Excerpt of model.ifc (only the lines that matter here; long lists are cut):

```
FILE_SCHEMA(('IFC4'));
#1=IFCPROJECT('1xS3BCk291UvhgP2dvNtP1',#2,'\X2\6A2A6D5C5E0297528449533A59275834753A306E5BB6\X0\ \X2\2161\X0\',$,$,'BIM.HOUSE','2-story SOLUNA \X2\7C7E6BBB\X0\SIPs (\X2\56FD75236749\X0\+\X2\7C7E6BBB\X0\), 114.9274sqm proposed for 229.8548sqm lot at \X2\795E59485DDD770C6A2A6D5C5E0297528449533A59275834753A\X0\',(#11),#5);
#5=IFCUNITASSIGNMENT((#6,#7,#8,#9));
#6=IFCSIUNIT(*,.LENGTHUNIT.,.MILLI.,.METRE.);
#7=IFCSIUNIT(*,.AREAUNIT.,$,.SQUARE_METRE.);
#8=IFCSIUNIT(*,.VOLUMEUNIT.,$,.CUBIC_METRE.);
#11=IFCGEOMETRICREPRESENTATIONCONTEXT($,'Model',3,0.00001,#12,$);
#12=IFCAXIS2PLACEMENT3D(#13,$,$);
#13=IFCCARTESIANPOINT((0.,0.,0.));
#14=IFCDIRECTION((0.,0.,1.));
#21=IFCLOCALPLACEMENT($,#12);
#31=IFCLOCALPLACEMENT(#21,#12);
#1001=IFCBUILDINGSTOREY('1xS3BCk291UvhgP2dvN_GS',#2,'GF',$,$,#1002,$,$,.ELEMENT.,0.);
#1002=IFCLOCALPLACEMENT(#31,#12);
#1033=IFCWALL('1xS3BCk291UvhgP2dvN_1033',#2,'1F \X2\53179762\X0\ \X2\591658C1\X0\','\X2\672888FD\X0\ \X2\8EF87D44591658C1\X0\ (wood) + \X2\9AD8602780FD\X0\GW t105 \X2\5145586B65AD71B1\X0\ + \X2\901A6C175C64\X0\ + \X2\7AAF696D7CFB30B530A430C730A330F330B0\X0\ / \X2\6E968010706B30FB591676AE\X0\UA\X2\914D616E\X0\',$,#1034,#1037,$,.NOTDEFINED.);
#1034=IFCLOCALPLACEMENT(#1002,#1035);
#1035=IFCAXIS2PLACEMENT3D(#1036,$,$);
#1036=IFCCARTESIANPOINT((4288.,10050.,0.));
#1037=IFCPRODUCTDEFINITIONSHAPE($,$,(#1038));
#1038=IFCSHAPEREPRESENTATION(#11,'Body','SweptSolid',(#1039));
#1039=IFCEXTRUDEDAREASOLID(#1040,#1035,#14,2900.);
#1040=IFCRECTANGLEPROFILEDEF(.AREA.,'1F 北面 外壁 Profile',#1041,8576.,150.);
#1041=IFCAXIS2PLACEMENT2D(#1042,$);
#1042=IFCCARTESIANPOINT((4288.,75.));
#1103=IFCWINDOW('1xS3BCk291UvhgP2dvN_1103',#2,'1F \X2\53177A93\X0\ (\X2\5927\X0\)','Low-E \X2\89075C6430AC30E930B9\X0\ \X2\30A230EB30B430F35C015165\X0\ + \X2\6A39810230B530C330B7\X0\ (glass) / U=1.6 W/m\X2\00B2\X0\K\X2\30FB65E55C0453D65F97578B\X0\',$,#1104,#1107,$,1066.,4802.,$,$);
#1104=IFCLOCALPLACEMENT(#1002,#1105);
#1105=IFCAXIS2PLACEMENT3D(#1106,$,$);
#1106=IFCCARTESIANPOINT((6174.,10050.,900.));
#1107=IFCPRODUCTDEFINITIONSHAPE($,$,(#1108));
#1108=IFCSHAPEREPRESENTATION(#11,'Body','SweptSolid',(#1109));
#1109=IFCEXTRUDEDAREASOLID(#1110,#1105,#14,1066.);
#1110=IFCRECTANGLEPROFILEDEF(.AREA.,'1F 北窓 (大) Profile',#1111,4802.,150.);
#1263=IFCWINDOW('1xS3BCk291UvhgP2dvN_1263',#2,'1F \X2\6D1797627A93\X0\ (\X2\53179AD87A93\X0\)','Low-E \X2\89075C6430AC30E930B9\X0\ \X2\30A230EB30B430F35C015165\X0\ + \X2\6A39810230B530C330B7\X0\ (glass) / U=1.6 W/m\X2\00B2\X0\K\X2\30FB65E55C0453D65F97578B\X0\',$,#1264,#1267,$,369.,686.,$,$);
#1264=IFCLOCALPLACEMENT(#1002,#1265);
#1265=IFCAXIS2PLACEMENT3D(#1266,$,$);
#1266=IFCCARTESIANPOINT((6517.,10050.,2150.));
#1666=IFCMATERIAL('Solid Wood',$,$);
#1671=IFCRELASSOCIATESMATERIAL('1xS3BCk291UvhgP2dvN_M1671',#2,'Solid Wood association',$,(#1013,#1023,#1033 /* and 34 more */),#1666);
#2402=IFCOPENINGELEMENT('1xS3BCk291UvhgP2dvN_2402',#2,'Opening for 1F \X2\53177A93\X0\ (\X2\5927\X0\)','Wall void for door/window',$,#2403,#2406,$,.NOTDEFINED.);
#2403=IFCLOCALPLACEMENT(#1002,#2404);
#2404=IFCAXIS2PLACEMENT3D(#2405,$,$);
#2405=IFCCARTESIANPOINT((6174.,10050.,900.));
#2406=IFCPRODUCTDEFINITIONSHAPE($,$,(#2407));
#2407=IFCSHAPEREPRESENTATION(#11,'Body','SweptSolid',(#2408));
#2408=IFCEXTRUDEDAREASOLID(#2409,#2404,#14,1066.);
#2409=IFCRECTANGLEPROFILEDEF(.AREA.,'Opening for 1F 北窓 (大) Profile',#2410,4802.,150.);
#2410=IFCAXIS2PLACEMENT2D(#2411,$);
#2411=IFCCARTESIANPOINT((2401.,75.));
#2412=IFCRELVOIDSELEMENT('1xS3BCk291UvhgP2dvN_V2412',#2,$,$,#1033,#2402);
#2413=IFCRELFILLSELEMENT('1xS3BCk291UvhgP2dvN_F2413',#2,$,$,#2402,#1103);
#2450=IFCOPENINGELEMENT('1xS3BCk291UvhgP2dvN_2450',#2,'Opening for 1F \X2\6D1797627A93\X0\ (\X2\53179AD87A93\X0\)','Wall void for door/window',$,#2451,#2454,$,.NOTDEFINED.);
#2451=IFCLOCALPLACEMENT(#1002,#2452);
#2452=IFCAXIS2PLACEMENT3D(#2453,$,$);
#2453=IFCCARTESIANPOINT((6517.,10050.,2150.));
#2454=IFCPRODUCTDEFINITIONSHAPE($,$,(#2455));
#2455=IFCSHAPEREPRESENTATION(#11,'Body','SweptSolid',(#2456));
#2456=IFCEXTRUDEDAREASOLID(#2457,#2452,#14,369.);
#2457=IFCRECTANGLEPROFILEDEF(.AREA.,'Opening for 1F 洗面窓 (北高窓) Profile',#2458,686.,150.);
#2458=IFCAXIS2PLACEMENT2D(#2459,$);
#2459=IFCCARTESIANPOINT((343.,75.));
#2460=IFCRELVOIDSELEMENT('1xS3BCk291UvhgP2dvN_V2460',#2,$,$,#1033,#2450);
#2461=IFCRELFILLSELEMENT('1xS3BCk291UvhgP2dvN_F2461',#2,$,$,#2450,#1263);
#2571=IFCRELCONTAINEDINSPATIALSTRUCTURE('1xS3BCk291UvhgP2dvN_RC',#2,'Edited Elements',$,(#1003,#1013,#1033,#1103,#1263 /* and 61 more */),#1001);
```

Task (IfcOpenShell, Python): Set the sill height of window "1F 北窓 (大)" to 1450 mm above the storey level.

```python
import numpy as np
import ifcopenshell
import ifcopenshell.api.geometry
import ifcopenshell.geom
import ifcopenshell.util.element
import ifcopenshell.util.placement
import ifcopenshell.util.shape
import ifcopenshell.util.unit

model = ifcopenshell.open("model.ifc")
unit_scale = ifcopenshell.util.unit.calculate_unit_scale(model)

window = model.by_guid("1xS3BCk291UvhgP2dvN_1103")
opening = window.FillsVoids[0].RelatingOpeningElement
storey = ifcopenshell.util.element.get_container(window, ifc_class="IfcBuildingStorey")
level = ifcopenshell.util.placement.get_local_placement(storey.ObjectPlacement)[2, 3]

# The opening's origin need not be at the sill, so measure its lowest point.
shape = ifcopenshell.geom.create_shape(ifcopenshell.geom.settings(), opening)
bottom = ifcopenshell.util.shape.get_shape_bottom_elevation(shape, shape.geometry) / unit_scale
dz = level + 1.45 / unit_scale - bottom

shift = np.array([0.0, 0.0, dz])
# The window is not placed relative to its opening, so move both.
for product in (opening, window):
    matrix = ifcopenshell.util.placement.get_local_placement(product.ObjectPlacement)
    matrix[:3, 3] += shift
    ifcopenshell.api.geometry.edit_object_placement(model, product=product, matrix=matrix, is_si=False)

print(f"moved by {dz * unit_scale:+.3f} m")

model.write("model-out.ifc")
```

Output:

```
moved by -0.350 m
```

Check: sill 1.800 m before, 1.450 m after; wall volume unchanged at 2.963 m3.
